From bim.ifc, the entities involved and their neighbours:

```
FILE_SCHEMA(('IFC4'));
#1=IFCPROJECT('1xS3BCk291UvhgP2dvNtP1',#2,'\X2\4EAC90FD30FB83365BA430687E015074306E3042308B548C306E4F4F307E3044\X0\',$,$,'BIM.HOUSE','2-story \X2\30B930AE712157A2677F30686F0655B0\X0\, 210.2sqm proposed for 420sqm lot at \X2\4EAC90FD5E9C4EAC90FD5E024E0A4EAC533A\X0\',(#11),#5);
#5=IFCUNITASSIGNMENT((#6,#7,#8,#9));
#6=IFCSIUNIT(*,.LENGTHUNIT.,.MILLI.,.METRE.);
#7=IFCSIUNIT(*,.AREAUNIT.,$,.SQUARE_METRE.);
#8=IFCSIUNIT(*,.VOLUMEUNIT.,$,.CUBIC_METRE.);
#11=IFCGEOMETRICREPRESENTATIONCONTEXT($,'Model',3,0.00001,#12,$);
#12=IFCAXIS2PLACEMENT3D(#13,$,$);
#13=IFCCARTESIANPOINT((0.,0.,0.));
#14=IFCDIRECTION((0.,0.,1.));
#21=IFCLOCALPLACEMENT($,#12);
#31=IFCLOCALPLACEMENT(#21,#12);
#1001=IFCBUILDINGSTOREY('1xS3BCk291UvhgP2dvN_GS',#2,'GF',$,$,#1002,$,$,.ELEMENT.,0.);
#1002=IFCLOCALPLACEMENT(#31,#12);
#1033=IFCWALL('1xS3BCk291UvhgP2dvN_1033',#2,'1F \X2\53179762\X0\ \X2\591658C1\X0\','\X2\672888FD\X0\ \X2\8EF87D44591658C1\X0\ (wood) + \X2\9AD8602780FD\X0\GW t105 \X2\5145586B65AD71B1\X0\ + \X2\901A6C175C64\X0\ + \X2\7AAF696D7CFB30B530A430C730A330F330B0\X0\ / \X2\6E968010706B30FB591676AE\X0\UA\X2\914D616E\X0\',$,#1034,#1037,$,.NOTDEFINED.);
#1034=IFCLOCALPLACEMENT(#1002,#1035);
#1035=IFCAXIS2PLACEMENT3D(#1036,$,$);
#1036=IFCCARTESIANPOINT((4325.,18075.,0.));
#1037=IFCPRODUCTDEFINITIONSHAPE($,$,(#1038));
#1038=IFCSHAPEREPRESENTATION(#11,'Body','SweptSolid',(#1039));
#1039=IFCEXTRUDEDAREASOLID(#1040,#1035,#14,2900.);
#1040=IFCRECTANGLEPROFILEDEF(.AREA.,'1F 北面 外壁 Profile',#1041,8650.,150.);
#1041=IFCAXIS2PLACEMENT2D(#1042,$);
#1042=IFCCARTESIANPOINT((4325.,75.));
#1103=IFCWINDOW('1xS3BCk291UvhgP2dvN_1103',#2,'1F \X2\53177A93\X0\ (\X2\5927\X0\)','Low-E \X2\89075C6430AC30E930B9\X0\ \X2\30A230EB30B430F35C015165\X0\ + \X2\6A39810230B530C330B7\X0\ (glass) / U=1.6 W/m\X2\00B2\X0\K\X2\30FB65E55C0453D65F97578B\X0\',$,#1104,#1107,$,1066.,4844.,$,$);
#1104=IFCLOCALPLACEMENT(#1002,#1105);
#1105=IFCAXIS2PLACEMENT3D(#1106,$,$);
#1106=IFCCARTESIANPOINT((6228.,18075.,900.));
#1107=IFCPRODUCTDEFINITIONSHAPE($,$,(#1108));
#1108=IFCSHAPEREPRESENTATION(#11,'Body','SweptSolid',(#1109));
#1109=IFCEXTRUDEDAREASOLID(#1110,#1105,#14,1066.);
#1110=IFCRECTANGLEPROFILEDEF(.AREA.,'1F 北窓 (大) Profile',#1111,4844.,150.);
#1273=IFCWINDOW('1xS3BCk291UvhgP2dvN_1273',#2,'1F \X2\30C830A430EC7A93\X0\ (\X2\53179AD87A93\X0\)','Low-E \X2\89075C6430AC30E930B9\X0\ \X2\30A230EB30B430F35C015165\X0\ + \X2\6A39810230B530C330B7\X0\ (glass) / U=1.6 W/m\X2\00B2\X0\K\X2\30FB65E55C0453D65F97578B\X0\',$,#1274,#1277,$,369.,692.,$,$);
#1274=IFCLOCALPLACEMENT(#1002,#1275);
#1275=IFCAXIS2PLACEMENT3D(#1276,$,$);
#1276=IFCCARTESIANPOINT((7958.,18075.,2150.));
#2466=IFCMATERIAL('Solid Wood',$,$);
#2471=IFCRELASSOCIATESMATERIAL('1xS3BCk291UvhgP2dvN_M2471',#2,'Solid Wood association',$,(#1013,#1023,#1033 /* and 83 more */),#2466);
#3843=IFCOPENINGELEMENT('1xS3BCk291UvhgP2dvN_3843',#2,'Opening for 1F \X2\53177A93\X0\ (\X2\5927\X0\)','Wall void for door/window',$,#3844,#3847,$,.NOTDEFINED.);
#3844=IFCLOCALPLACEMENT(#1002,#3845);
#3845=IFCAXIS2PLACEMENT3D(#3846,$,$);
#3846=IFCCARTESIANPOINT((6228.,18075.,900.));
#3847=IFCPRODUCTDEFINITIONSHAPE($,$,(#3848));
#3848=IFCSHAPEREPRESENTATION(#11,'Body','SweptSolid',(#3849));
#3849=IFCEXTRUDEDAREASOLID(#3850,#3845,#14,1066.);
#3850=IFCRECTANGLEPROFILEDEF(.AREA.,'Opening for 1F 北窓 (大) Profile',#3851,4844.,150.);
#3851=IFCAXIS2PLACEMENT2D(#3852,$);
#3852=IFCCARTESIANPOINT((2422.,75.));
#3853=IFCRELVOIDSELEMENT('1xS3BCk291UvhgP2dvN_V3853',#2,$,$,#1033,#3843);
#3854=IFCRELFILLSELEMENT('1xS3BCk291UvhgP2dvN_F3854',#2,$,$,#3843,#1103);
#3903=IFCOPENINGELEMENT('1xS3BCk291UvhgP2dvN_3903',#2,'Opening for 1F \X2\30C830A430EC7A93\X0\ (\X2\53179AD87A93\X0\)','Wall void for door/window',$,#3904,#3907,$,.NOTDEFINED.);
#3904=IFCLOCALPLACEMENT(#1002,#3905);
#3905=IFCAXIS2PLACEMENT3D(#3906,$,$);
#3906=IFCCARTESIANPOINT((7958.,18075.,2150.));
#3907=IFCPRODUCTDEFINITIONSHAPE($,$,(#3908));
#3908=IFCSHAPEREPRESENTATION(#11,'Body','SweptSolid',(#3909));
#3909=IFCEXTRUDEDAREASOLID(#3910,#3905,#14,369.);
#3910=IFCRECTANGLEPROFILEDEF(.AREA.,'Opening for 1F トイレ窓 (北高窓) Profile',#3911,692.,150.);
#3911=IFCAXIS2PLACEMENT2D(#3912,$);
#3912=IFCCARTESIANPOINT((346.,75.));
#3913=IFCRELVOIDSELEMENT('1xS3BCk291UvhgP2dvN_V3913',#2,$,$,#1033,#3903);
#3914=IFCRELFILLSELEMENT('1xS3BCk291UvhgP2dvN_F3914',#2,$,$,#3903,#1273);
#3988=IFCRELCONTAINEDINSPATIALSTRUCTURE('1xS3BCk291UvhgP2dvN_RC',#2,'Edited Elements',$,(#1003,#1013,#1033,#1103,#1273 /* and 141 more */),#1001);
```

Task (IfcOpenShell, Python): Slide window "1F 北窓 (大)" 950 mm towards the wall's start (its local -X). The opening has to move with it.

```python
import ifcopenshell
import ifcopenshell.api.geometry
import ifcopenshell.util.placement
import ifcopenshell.util.unit

model = ifcopenshell.open("bim.ifc")
unit_scale = ifcopenshell.util.unit.calculate_unit_scale(model)

window = model.by_guid("1xS3BCk291UvhgP2dvN_1103")
opening = window.FillsVoids[0].RelatingOpeningElement
wall = opening.VoidsElements[0].RelatingBuildingElement

wall_matrix = ifcopenshell.util.placement.get_local_placement(wall.ObjectPlacement)
shift = wall_matrix[:3, 0] * -0.95 / unit_scale
before = ifcopenshell.util.placement.get_local_placement(window.ObjectPlacement)[:3, 3].copy()

# The window is not placed relative to its opening, so move both.
for product in (opening, window):
    matrix = ifcopenshell.util.placement.get_local_placement(product.ObjectPlacement)
    matrix[:3, 3] += shift
    ifcopenshell.api.geometry.edit_object_placement(model, product=product, matrix=matrix, is_si=False)

after = ifcopenshell.util.placement.get_local_placement(window.ObjectPlacement)[:3, 3]
print("window moved by", (after - before).round(3) + 0.0)

model.write("bim_rev.ifc")
```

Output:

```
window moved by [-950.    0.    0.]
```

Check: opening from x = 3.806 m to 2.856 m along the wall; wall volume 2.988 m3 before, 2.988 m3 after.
